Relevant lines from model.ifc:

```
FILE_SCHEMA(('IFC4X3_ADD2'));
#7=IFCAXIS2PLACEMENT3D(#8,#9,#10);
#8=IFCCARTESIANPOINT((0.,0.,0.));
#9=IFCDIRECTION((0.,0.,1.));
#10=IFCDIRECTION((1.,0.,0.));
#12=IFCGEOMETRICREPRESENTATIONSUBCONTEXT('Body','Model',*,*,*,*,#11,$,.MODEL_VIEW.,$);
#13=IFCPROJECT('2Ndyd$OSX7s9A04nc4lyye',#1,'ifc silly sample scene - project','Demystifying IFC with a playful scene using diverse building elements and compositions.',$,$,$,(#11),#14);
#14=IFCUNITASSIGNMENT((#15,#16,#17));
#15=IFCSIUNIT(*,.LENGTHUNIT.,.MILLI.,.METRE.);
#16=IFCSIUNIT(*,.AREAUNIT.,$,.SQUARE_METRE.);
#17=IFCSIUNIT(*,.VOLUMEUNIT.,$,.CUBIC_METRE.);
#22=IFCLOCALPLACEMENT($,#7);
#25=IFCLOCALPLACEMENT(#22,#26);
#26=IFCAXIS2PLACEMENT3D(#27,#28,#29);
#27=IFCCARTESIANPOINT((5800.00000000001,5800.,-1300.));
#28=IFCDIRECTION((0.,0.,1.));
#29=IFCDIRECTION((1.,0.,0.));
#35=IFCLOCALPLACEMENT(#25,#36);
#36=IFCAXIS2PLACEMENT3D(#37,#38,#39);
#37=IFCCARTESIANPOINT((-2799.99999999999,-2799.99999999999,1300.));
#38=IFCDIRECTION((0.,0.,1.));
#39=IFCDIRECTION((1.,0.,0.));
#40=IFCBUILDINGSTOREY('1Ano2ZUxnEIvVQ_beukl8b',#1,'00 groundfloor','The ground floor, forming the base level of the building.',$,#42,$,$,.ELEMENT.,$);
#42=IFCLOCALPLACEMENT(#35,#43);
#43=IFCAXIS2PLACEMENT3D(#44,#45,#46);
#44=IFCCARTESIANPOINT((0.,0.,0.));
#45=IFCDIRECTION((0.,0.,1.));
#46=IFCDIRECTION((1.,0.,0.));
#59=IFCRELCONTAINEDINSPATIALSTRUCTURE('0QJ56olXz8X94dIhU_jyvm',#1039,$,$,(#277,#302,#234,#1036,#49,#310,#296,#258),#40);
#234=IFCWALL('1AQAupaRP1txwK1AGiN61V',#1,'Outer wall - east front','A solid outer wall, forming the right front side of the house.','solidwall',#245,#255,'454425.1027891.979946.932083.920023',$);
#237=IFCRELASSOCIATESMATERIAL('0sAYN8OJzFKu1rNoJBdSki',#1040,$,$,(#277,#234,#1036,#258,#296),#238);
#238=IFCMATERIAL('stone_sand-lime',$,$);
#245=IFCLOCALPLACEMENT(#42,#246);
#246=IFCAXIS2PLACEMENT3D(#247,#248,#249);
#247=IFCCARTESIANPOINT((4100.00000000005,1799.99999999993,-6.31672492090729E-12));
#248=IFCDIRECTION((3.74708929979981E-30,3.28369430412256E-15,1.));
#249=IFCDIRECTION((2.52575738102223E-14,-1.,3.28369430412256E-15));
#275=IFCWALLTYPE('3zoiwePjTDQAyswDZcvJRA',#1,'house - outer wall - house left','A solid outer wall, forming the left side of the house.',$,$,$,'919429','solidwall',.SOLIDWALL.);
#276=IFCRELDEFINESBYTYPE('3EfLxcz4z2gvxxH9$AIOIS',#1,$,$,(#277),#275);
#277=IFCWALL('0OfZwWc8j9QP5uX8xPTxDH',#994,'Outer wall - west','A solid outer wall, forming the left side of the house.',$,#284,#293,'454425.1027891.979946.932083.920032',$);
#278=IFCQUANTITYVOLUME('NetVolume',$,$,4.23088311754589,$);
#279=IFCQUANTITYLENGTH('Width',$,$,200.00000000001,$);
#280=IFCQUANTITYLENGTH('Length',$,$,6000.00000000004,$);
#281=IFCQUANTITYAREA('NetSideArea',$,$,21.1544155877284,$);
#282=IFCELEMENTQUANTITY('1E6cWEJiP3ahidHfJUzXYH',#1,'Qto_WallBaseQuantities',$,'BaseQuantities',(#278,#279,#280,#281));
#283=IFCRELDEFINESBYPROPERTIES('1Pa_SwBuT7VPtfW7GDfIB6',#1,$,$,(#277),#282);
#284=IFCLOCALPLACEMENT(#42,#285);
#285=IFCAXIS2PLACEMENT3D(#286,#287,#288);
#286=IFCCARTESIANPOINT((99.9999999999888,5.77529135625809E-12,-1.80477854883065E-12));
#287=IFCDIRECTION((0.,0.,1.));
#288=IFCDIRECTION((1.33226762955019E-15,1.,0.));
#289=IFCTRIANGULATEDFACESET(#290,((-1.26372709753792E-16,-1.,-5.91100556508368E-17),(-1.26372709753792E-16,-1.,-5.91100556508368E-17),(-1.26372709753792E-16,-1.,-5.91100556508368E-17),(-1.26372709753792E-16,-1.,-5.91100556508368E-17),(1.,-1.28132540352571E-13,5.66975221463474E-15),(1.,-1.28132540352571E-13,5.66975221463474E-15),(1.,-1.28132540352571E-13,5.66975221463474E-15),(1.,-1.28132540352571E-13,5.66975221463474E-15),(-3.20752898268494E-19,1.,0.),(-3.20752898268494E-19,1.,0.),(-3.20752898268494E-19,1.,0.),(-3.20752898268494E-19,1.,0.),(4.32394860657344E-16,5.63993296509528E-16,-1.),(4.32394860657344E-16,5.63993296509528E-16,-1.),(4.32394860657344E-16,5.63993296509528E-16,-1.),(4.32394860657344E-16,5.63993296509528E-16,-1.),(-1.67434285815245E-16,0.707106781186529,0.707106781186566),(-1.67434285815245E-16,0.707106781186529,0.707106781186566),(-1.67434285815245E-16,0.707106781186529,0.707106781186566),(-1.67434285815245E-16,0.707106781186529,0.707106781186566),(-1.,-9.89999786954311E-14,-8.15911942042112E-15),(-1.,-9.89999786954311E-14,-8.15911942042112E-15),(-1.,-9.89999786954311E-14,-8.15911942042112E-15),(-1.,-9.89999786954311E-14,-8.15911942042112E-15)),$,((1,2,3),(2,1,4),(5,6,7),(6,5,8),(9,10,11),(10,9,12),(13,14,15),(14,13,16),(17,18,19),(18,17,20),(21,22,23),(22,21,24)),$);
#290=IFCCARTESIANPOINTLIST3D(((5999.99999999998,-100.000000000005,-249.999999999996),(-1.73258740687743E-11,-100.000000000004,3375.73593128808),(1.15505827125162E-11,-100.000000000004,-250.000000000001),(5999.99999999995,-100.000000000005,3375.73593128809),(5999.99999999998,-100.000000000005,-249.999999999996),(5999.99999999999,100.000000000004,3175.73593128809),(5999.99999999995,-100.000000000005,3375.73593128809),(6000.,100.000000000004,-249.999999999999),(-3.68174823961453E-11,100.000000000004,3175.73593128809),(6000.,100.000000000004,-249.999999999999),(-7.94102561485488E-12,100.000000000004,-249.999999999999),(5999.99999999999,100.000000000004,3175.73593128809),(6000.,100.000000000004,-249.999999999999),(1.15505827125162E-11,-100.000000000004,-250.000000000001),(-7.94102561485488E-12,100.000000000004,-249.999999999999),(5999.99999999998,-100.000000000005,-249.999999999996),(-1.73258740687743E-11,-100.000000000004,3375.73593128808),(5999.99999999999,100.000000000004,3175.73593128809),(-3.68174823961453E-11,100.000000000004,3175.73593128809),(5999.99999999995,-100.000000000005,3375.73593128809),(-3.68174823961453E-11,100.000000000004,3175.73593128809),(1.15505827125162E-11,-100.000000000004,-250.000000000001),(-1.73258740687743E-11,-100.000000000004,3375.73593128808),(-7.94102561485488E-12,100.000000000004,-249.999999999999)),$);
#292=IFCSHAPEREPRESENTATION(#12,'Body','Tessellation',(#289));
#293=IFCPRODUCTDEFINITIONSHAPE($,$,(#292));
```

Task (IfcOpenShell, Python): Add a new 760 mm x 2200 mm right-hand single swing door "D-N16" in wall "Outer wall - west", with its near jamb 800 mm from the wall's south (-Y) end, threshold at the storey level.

```python
import numpy as np
import ifcopenshell
import ifcopenshell.api.feature
import ifcopenshell.api.geometry
import ifcopenshell.api.pset
import ifcopenshell.api.root
import ifcopenshell.api.spatial
import ifcopenshell.geom
import ifcopenshell.util.element
import ifcopenshell.util.placement
import ifcopenshell.util.representation
import ifcopenshell.util.shape
import ifcopenshell.util.unit

model = ifcopenshell.open("model.ifc")
unit_scale = ifcopenshell.util.unit.calculate_unit_scale(model)
area_scale = ifcopenshell.util.unit.calculate_unit_scale(model, "AREAUNIT")
volume_scale = ifcopenshell.util.unit.calculate_unit_scale(model, "VOLUMEUNIT")
settings = ifcopenshell.geom.settings()


def volume(element):
    """Net volume in cubic metres, openings subtracted."""
    shape = ifcopenshell.geom.create_shape(settings, element)
    return ifcopenshell.util.shape.get_volume(shape.geometry)


wall = model.by_guid("0OfZwWc8j9QP5uX8xPTxDH")
storey = ifcopenshell.util.element.get_container(wall, ifc_class="IfcBuildingStorey")
context = ifcopenshell.util.representation.get_context(model, "Model", "Body", "MODEL_VIEW")
before = volume(wall)

width, height, from_end, sill = 0.76, 2.2, 0.8, 0.0  # metres

# The wall runs along its own X axis, and the end named is its -X end.
wall_shape = ifcopenshell.geom.create_shape(settings, wall)
x, y, z = ifcopenshell.util.shape.get_vertices(wall_shape.geometry).T
start = x.min() + from_end
face, thickness = float(y.min()), float(y.max() - y.min())
wall_matrix = ifcopenshell.util.placement.get_local_placement(wall.ObjectPlacement)
level = ifcopenshell.util.placement.get_local_placement(storey.ObjectPlacement)[2, 3]


def in_wall(x, y):
    """Placement at x, y metres in the wall's axes, at sill height."""
    matrix = wall_matrix.copy()
    matrix[:, 3] = wall_matrix @ np.array([x / unit_scale, y / unit_scale, 0.0, 1.0])
    matrix[2, 3] = level + sill / unit_scale
    return matrix


# Opening: a box that overshoots both wall faces by 50 mm.
opening = ifcopenshell.api.root.create_entity(model, ifc_class="IfcOpeningElement", predefined_type="OPENING")
box = ifcopenshell.api.geometry.add_wall_representation(
    model, context=context, length=width, height=height, thickness=thickness + 0.1
)
ifcopenshell.api.geometry.assign_representation(model, product=opening, representation=box)
ifcopenshell.api.geometry.edit_object_placement(model, product=opening, matrix=in_wall(start, face - 0.05), is_si=False)
ifcopenshell.api.feature.add_feature(model, feature=opening, element=wall)

door = ifcopenshell.api.root.create_entity(model, ifc_class="IfcDoor", name="D-N16", predefined_type="DOOR")
door.OverallWidth, door.OverallHeight = width / unit_scale, height / unit_scale
door.OperationType = "SINGLE_SWING_RIGHT"
body = ifcopenshell.api.geometry.add_door_representation(
    model,
    context=context,
    overall_width=door.OverallWidth,
    overall_height=door.OverallHeight,
    operation_type="SINGLE_SWING_RIGHT",
    lining_properties={"LiningDepth": thickness / unit_scale, "ThresholdDepth": thickness / unit_scale},
)
ifcopenshell.api.geometry.assign_representation(model, product=door, representation=body)
ifcopenshell.api.spatial.assign_container(model, products=[door], relating_structure=storey)
ifcopenshell.api.feature.add_filling(model, opening=opening, element=door)

# The lining spans the wall, so the door starts at the wall face.
ifcopenshell.api.geometry.edit_object_placement(model, product=door, matrix=in_wall(start, face), is_si=False)

after = volume(wall)

# Update the wall's stored quantities.
qto = model.by_id(ifcopenshell.util.element.get_pset(wall, "Qto_WallBaseQuantities", should_inherit=False)["id"])
ifcopenshell.api.pset.edit_qto(model, qto=qto, properties={
    "NetVolume": after / volume_scale,
    "NetSideArea": after / thickness / area_scale,
})

print(f"wall volume {before:.3f} -> {after:.3f} m3")

model.write("model-out.ifc")
```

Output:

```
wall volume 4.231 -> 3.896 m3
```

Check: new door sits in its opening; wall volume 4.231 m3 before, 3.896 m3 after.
